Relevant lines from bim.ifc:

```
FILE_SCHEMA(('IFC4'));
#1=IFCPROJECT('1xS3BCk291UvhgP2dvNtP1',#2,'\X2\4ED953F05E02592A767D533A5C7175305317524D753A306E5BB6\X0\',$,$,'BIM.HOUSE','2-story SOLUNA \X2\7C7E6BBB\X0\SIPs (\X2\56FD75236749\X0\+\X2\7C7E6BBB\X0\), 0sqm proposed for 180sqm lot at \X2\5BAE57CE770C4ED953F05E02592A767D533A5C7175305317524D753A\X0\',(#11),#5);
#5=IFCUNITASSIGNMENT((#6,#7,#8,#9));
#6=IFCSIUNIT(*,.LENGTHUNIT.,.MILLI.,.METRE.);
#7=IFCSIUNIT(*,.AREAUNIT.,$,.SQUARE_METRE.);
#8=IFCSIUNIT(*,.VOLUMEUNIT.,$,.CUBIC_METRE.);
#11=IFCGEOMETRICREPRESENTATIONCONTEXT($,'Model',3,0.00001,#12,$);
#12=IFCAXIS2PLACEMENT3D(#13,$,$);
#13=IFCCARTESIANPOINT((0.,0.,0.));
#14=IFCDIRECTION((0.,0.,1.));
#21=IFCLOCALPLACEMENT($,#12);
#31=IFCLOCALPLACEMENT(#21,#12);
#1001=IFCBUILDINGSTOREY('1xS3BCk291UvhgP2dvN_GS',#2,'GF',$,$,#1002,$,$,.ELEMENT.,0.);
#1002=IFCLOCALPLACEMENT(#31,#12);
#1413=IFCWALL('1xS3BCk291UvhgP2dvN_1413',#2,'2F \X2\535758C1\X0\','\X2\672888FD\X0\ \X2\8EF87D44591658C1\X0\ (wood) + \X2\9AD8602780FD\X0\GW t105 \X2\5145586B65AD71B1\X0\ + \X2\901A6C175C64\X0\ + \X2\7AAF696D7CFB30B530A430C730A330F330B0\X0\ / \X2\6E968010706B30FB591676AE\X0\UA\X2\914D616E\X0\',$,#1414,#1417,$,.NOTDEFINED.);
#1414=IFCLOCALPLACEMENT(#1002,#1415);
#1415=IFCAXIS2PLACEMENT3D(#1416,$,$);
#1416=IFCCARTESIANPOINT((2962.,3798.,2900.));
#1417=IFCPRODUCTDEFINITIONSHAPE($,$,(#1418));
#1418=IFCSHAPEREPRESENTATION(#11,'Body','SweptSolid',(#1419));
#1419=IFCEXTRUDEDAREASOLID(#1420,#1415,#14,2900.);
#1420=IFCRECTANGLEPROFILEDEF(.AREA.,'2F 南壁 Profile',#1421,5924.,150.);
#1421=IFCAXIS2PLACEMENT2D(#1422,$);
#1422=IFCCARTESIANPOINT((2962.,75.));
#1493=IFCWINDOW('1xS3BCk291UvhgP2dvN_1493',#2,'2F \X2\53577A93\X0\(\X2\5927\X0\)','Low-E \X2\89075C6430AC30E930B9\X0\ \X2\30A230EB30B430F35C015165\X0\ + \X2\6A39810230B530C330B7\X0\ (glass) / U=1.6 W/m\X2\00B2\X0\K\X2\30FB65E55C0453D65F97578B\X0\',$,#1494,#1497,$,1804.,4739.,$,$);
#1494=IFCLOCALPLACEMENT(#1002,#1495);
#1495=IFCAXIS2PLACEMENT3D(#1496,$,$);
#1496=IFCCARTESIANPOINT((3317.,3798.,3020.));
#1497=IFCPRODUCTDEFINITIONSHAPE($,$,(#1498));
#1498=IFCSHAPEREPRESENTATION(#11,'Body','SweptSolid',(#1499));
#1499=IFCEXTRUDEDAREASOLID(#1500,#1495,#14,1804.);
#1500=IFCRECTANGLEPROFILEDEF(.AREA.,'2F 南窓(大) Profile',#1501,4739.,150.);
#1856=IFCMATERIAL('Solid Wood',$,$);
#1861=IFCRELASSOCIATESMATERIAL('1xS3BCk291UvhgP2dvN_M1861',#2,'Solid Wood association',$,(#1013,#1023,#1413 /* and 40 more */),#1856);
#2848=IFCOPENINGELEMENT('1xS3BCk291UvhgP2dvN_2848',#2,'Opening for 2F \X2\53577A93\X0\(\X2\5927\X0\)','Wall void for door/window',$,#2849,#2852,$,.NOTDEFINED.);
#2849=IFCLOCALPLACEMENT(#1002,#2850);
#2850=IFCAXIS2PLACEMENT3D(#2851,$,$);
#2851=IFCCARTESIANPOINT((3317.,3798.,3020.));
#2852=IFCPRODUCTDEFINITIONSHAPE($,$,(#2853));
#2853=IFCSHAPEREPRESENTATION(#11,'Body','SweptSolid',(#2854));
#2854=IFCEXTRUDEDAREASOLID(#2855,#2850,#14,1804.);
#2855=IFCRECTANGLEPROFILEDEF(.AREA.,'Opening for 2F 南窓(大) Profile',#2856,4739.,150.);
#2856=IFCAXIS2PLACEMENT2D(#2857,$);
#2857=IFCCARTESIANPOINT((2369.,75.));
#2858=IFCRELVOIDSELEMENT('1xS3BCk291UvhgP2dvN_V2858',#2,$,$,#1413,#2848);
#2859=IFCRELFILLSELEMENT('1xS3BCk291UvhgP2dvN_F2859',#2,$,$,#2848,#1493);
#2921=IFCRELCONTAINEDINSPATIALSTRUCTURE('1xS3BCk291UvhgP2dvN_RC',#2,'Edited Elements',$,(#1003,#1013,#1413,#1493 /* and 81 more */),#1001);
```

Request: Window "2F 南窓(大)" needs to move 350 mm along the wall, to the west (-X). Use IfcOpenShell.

```python
import ifcopenshell
import ifcopenshell.api.geometry
import ifcopenshell.util.placement

model = ifcopenshell.open("bim.ifc")

window = model.by_guid("1xS3BCk291UvhgP2dvN_1493")
opening = window.FillsVoids[0].RelatingOpeningElement
wall = opening.VoidsElements[0].RelatingBuildingElement

wall_matrix = ifcopenshell.util.placement.get_local_placement(wall.ObjectPlacement)
shift = wall_matrix[:3, 0] * -350.0
before = ifcopenshell.util.placement.get_local_placement(window.ObjectPlacement)[:3, 3].copy()

# The window is not placed relative to its opening, so move both.
for product in (opening, window):
    matrix = ifcopenshell.util.placement.get_local_placement(product.ObjectPlacement)
    matrix[:3, 3] += shift
    ifcopenshell.api.geometry.edit_object_placement(model, product=product, matrix=matrix, is_si=False)

after = ifcopenshell.util.placement.get_local_placement(window.ObjectPlacement)[:3, 3]
print("window moved by", (after - before).round(3) + 0.0)

model.write("bim-out.ifc")
```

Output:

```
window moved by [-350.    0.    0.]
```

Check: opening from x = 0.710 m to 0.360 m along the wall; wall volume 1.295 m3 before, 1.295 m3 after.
